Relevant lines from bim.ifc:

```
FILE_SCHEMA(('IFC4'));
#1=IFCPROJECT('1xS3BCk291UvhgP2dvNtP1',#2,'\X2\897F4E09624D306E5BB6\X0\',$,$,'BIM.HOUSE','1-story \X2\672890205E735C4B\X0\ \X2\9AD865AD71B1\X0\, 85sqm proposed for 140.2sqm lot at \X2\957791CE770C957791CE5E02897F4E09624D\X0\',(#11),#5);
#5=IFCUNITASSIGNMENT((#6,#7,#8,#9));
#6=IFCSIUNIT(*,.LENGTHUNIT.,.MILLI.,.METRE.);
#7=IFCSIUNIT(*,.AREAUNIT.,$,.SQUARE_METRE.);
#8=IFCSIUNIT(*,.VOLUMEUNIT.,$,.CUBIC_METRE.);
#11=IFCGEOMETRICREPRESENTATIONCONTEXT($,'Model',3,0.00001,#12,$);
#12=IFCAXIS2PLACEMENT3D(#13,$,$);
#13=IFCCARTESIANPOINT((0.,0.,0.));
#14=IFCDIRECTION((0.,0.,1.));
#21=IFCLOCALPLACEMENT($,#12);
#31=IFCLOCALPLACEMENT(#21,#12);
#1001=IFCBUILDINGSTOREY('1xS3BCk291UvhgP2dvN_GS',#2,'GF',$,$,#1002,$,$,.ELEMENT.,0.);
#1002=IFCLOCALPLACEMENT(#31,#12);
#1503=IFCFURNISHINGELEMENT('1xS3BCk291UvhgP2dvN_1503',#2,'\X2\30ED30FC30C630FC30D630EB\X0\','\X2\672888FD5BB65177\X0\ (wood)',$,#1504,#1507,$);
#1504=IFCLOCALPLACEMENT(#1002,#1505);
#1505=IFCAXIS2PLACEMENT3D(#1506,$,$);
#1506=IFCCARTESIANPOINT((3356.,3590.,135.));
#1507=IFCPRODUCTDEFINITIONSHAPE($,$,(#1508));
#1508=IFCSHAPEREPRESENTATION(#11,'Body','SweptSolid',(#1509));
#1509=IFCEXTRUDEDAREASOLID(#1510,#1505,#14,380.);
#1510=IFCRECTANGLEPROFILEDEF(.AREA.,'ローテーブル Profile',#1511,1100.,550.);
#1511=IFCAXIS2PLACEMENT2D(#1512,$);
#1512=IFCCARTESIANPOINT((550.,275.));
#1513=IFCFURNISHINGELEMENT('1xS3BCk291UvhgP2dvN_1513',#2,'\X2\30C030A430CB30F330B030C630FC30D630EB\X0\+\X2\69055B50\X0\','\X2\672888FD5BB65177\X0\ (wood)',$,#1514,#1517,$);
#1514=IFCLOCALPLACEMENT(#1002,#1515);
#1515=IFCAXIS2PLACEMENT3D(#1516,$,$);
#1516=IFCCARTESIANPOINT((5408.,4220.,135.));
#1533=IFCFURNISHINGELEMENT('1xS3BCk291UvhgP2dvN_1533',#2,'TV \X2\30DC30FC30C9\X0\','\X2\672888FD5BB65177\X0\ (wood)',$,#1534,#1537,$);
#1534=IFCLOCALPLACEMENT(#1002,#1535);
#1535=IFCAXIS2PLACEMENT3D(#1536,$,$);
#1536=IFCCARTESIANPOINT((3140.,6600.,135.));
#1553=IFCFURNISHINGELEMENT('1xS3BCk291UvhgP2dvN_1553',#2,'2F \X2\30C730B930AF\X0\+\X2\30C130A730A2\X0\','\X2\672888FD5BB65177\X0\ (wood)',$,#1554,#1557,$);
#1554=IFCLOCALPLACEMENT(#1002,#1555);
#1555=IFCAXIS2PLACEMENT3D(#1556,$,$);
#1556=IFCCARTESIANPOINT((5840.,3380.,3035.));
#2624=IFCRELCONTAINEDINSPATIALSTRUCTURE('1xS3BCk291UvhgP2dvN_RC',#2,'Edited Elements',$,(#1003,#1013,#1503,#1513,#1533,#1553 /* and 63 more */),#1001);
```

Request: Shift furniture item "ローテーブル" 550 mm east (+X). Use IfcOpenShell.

```python
import ifcopenshell
import ifcopenshell.api.geometry
import ifcopenshell.util.placement
import ifcopenshell.util.unit

model = ifcopenshell.open("bim.ifc")
unit_scale = ifcopenshell.util.unit.calculate_unit_scale(model)

item = model.by_guid("1xS3BCk291UvhgP2dvN_1503")
matrix = ifcopenshell.util.placement.get_local_placement(item.ObjectPlacement)
matrix[0, 3] += 0.55 / unit_scale
ifcopenshell.api.geometry.edit_object_placement(model, product=item, matrix=matrix, is_si=False)

print(ifcopenshell.util.placement.get_local_placement(item.ObjectPlacement).round(3) + 0.0)

model.write("bim_rev.ifc")
```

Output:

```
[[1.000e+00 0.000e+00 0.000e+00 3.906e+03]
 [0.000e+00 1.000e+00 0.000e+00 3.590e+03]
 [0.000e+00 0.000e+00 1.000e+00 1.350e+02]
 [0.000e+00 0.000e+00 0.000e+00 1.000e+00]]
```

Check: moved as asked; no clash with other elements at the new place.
